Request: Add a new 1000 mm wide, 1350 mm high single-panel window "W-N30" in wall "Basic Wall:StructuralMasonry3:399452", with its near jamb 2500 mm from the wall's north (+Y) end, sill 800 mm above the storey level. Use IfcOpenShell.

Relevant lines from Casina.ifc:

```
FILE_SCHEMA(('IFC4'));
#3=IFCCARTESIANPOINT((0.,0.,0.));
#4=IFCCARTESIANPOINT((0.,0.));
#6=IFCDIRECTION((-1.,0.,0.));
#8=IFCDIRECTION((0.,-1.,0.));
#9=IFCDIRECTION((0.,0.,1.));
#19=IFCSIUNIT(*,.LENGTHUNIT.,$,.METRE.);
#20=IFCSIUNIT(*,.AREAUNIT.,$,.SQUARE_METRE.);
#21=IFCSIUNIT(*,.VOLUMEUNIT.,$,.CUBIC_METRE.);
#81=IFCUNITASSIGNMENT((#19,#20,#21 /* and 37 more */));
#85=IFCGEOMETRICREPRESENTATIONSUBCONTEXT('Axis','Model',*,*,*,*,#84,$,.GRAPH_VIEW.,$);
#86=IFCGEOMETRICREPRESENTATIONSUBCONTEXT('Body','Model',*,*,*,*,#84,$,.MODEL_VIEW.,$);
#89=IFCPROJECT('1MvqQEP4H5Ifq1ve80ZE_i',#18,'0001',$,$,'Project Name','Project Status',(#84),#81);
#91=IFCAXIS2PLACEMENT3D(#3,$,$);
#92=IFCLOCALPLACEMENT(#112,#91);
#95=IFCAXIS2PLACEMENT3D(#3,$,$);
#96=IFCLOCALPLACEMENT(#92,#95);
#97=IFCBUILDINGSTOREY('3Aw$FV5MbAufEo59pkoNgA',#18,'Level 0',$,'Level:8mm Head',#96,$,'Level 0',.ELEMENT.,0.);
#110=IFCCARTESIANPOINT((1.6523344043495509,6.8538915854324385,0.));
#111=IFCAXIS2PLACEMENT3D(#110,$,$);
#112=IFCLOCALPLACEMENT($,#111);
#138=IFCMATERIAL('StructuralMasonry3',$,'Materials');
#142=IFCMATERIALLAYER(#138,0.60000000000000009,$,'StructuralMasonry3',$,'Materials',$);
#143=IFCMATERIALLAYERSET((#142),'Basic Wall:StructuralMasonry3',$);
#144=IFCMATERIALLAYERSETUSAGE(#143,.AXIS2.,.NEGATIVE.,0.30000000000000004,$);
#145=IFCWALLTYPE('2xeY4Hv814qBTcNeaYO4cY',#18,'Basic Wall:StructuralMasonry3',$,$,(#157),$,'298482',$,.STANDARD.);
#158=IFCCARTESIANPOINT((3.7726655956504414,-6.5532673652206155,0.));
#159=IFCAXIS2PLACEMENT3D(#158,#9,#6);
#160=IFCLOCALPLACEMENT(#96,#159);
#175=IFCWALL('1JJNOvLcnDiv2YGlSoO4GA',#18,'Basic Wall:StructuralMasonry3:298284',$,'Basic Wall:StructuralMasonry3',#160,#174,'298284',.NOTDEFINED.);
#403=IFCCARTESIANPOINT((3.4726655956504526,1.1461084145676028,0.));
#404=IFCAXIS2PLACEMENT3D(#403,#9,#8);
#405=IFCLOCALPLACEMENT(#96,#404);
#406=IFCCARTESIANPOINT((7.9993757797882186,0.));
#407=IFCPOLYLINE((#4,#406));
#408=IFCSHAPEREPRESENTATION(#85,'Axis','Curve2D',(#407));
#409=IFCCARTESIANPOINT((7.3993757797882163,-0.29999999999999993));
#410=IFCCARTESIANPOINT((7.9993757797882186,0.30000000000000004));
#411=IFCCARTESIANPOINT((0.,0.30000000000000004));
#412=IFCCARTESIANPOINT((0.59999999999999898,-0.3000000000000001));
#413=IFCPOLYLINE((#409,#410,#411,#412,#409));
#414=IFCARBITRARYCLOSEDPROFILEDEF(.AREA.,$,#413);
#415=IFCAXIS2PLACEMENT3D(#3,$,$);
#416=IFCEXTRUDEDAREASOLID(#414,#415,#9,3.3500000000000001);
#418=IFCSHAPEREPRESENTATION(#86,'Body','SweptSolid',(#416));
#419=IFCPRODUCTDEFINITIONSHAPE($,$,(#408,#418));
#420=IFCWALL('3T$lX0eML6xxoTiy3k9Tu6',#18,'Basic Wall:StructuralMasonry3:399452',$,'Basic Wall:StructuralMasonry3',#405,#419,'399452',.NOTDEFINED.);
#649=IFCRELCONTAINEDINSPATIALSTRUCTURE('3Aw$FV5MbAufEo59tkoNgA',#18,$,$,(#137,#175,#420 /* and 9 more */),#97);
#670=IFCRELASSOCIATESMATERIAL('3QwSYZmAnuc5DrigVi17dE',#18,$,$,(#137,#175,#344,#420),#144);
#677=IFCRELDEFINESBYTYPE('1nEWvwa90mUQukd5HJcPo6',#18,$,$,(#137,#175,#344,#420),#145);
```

```python
import numpy as np
import ifcopenshell
import ifcopenshell.api.feature
import ifcopenshell.api.geometry
import ifcopenshell.api.root
import ifcopenshell.api.spatial
import ifcopenshell.geom
import ifcopenshell.util.element
import ifcopenshell.util.placement
import ifcopenshell.util.representation
import ifcopenshell.util.shape
import ifcopenshell.util.unit

model = ifcopenshell.open("Casina.ifc")
unit_scale = ifcopenshell.util.unit.calculate_unit_scale(model)
settings = ifcopenshell.geom.settings()


def volume(element):
    """Net volume in cubic metres, openings subtracted."""
    shape = ifcopenshell.geom.create_shape(settings, element)
    return ifcopenshell.util.shape.get_volume(shape.geometry)


wall = model.by_guid("3T$lX0eML6xxoTiy3k9Tu6")
storey = ifcopenshell.util.element.get_container(wall, ifc_class="IfcBuildingStorey")
context = ifcopenshell.util.representation.get_context(model, "Model", "Body", "MODEL_VIEW")
before = volume(wall)

width, height, from_end, sill = 1, 1.35, 2.5, 0.8  # metres

# The wall runs along its own X axis, and the end named is its -X end.
wall_shape = ifcopenshell.geom.create_shape(settings, wall)
x, y, z = ifcopenshell.util.shape.get_vertices(wall_shape.geometry).T
start = x.min() + from_end
face, thickness = float(y.min()), float(y.max() - y.min())
wall_matrix = ifcopenshell.util.placement.get_local_placement(wall.ObjectPlacement)
level = ifcopenshell.util.placement.get_local_placement(storey.ObjectPlacement)[2, 3]


def in_wall(x, y):
    """Placement at x, y metres in the wall's axes, at sill height."""
    matrix = wall_matrix.copy()
    matrix[:, 3] = wall_matrix @ np.array([x / unit_scale, y / unit_scale, 0.0, 1.0])
    matrix[2, 3] = level + sill / unit_scale
    return matrix


# Opening: a box that overshoots both wall faces by 50 mm.
opening = ifcopenshell.api.root.create_entity(model, ifc_class="IfcOpeningElement", predefined_type="OPENING")
box = ifcopenshell.api.geometry.add_wall_representation(
    model, context=context, length=width, height=height, thickness=thickness + 0.1
)
ifcopenshell.api.geometry.assign_representation(model, product=opening, representation=box)
ifcopenshell.api.geometry.edit_object_placement(model, product=opening, matrix=in_wall(start, face - 0.05), is_si=False)
ifcopenshell.api.feature.add_feature(model, feature=opening, element=wall)

window = ifcopenshell.api.root.create_entity(model, ifc_class="IfcWindow", name="W-N30", predefined_type="WINDOW")
window.OverallWidth, window.OverallHeight = width / unit_scale, height / unit_scale
window.PartitioningType = "SINGLE_PANEL"
body = ifcopenshell.api.geometry.add_window_representation(
    model,
    context=context,
    overall_width=window.OverallWidth,
    overall_height=window.OverallHeight,
    partition_type="SINGLE_PANEL",
)
ifcopenshell.api.geometry.assign_representation(model, product=window, representation=body)
ifcopenshell.api.spatial.assign_container(model, products=[window], relating_structure=storey)
ifcopenshell.api.feature.add_filling(model, opening=opening, element=window)

# Centre the window in the wall's thickness.
ifcopenshell.api.geometry.edit_object_placement(model, product=window, matrix=in_wall(start, face), is_si=False)
window_shape = ifcopenshell.geom.create_shape(settings, window)
depth = ifcopenshell.util.shape.get_vertices(window_shape.geometry)[:, 1]
offset = face + thickness / 2 - (depth.min() + depth.max()) / 2
ifcopenshell.api.geometry.edit_object_placement(model, product=window, matrix=in_wall(start, offset), is_si=False)

after = volume(wall)

print(f"wall volume {before:.3f} -> {after:.3f} m3")

model.write("Casina-out.ifc")
```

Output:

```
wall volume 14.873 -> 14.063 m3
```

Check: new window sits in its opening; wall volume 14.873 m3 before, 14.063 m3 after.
